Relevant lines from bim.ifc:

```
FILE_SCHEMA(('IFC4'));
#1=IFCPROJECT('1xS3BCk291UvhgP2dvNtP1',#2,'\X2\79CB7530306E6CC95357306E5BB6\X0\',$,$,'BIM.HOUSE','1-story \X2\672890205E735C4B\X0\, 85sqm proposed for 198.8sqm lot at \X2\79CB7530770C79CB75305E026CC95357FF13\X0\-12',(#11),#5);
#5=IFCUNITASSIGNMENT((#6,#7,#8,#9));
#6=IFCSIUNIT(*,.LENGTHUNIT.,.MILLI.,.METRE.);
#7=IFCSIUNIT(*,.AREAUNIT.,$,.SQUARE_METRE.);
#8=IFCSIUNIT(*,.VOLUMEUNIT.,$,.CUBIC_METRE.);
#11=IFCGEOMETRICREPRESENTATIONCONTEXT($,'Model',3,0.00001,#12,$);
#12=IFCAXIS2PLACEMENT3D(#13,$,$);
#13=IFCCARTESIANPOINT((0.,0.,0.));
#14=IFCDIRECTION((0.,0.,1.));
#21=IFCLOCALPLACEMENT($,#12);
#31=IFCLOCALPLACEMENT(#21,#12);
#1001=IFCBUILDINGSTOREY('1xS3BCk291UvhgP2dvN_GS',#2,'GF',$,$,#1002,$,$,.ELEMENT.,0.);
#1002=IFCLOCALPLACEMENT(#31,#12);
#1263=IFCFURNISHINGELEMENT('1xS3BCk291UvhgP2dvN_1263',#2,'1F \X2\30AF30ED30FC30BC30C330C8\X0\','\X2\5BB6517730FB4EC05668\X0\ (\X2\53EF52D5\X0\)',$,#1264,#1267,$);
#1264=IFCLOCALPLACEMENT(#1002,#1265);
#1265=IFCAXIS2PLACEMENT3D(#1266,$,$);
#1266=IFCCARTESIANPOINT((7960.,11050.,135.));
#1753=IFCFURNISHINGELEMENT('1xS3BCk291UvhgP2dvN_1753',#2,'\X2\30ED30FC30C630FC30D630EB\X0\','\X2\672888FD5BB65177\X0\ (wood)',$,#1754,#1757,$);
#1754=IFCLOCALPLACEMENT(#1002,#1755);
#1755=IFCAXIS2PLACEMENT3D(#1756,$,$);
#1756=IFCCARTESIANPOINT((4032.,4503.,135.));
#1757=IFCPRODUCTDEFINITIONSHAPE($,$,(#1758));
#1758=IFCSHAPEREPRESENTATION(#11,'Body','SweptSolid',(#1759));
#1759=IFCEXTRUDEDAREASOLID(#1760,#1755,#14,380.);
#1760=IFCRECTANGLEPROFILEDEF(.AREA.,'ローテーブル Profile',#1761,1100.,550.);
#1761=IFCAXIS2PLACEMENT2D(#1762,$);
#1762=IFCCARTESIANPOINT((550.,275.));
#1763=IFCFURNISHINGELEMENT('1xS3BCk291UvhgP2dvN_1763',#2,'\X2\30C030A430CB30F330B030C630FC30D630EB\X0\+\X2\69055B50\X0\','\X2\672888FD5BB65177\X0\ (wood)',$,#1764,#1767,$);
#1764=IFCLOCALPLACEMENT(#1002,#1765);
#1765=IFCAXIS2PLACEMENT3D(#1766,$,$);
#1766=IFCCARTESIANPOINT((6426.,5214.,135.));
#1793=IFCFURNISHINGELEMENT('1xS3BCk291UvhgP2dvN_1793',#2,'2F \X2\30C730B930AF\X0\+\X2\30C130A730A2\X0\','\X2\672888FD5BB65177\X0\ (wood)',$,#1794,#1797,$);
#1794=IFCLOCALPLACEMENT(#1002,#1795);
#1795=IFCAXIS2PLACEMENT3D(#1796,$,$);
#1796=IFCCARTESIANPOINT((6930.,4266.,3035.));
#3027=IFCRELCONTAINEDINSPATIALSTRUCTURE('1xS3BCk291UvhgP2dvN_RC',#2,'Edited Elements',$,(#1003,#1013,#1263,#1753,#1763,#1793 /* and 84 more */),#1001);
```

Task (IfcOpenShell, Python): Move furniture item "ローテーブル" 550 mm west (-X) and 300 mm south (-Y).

```python
import ifcopenshell
import ifcopenshell.api.geometry
import ifcopenshell.util.placement
import ifcopenshell.util.unit

model = ifcopenshell.open("bim.ifc")
unit_scale = ifcopenshell.util.unit.calculate_unit_scale(model)

item = model.by_id(1753)
matrix = ifcopenshell.util.placement.get_local_placement(item.ObjectPlacement)
matrix[0, 3] -= 0.55 / unit_scale
matrix[1, 3] -= 0.3 / unit_scale
ifcopenshell.api.geometry.edit_object_placement(model, product=item, matrix=matrix, is_si=False)

print(ifcopenshell.util.placement.get_local_placement(item.ObjectPlacement).round(3) + 0.0)

model.write("bim_edited.ifc")
```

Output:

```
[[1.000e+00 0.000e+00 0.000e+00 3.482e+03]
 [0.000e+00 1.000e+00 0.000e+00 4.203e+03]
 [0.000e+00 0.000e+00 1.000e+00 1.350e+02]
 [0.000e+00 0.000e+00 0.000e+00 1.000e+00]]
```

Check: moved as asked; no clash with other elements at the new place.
